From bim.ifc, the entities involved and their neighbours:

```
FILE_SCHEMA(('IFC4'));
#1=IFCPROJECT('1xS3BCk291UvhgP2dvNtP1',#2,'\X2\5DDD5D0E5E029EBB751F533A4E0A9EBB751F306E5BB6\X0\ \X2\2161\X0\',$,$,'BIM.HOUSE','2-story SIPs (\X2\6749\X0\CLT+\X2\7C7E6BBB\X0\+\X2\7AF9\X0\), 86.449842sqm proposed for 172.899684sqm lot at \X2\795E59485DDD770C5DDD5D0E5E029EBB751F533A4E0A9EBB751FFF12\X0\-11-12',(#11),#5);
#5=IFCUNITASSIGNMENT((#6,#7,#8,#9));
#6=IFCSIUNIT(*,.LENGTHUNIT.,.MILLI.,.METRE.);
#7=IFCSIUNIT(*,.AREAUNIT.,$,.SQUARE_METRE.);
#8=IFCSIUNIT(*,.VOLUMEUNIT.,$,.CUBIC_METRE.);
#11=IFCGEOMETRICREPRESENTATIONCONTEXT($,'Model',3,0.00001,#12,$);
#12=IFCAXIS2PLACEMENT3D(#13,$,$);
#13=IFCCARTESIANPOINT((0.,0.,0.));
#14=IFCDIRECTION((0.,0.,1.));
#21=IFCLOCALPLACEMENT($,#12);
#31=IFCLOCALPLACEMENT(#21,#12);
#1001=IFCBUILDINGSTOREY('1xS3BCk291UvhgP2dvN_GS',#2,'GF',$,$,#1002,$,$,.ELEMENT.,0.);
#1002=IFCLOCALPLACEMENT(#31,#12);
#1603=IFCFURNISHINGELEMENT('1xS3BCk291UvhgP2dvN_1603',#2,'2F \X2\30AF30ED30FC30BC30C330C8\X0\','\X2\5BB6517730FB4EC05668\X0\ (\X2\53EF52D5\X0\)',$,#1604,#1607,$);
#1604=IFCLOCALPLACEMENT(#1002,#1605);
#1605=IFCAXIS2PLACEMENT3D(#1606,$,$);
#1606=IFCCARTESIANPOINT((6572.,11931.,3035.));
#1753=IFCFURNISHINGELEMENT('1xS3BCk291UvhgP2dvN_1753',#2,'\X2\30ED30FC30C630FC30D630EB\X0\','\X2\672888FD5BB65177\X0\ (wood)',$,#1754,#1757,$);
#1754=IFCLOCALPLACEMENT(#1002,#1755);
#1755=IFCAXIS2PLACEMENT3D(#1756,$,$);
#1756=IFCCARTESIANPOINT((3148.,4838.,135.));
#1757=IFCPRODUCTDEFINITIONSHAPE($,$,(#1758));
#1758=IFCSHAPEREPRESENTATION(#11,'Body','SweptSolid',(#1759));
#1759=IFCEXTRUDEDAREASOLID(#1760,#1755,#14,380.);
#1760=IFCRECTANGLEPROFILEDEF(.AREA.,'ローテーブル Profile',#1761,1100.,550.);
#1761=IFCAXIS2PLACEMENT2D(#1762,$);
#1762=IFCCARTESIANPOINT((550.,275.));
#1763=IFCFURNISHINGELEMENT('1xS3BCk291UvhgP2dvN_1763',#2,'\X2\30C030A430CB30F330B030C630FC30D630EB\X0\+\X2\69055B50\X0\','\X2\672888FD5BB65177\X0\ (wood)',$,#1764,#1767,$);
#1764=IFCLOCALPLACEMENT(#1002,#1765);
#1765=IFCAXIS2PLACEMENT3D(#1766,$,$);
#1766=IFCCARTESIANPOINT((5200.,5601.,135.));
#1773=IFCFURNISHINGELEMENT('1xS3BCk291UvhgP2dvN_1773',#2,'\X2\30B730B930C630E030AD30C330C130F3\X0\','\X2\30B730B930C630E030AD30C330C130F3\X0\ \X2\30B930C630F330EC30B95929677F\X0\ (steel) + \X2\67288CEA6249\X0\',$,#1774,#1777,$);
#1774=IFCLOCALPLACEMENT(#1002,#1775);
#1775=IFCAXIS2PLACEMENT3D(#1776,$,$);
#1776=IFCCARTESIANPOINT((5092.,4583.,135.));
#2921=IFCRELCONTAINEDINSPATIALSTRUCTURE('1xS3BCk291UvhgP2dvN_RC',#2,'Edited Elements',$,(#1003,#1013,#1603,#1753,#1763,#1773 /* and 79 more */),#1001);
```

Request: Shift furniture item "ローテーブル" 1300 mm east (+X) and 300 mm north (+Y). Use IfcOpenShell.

```python
import ifcopenshell
import ifcopenshell.api.geometry
import ifcopenshell.util.placement
import ifcopenshell.util.unit

model = ifcopenshell.open("bim.ifc")
unit_scale = ifcopenshell.util.unit.calculate_unit_scale(model)

item = model.by_guid("1xS3BCk291UvhgP2dvN_1753")
matrix = ifcopenshell.util.placement.get_local_placement(item.ObjectPlacement)
matrix[0, 3] += 1.3 / unit_scale
matrix[1, 3] += 0.3 / unit_scale
ifcopenshell.api.geometry.edit_object_placement(model, product=item, matrix=matrix, is_si=False)

print(ifcopenshell.util.placement.get_local_placement(item.ObjectPlacement).round(3) + 0.0)

model.write("bim_rev.ifc")
```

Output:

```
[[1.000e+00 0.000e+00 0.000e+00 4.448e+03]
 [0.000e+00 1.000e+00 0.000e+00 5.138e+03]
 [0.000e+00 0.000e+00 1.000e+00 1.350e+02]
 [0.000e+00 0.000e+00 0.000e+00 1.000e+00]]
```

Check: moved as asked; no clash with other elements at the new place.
